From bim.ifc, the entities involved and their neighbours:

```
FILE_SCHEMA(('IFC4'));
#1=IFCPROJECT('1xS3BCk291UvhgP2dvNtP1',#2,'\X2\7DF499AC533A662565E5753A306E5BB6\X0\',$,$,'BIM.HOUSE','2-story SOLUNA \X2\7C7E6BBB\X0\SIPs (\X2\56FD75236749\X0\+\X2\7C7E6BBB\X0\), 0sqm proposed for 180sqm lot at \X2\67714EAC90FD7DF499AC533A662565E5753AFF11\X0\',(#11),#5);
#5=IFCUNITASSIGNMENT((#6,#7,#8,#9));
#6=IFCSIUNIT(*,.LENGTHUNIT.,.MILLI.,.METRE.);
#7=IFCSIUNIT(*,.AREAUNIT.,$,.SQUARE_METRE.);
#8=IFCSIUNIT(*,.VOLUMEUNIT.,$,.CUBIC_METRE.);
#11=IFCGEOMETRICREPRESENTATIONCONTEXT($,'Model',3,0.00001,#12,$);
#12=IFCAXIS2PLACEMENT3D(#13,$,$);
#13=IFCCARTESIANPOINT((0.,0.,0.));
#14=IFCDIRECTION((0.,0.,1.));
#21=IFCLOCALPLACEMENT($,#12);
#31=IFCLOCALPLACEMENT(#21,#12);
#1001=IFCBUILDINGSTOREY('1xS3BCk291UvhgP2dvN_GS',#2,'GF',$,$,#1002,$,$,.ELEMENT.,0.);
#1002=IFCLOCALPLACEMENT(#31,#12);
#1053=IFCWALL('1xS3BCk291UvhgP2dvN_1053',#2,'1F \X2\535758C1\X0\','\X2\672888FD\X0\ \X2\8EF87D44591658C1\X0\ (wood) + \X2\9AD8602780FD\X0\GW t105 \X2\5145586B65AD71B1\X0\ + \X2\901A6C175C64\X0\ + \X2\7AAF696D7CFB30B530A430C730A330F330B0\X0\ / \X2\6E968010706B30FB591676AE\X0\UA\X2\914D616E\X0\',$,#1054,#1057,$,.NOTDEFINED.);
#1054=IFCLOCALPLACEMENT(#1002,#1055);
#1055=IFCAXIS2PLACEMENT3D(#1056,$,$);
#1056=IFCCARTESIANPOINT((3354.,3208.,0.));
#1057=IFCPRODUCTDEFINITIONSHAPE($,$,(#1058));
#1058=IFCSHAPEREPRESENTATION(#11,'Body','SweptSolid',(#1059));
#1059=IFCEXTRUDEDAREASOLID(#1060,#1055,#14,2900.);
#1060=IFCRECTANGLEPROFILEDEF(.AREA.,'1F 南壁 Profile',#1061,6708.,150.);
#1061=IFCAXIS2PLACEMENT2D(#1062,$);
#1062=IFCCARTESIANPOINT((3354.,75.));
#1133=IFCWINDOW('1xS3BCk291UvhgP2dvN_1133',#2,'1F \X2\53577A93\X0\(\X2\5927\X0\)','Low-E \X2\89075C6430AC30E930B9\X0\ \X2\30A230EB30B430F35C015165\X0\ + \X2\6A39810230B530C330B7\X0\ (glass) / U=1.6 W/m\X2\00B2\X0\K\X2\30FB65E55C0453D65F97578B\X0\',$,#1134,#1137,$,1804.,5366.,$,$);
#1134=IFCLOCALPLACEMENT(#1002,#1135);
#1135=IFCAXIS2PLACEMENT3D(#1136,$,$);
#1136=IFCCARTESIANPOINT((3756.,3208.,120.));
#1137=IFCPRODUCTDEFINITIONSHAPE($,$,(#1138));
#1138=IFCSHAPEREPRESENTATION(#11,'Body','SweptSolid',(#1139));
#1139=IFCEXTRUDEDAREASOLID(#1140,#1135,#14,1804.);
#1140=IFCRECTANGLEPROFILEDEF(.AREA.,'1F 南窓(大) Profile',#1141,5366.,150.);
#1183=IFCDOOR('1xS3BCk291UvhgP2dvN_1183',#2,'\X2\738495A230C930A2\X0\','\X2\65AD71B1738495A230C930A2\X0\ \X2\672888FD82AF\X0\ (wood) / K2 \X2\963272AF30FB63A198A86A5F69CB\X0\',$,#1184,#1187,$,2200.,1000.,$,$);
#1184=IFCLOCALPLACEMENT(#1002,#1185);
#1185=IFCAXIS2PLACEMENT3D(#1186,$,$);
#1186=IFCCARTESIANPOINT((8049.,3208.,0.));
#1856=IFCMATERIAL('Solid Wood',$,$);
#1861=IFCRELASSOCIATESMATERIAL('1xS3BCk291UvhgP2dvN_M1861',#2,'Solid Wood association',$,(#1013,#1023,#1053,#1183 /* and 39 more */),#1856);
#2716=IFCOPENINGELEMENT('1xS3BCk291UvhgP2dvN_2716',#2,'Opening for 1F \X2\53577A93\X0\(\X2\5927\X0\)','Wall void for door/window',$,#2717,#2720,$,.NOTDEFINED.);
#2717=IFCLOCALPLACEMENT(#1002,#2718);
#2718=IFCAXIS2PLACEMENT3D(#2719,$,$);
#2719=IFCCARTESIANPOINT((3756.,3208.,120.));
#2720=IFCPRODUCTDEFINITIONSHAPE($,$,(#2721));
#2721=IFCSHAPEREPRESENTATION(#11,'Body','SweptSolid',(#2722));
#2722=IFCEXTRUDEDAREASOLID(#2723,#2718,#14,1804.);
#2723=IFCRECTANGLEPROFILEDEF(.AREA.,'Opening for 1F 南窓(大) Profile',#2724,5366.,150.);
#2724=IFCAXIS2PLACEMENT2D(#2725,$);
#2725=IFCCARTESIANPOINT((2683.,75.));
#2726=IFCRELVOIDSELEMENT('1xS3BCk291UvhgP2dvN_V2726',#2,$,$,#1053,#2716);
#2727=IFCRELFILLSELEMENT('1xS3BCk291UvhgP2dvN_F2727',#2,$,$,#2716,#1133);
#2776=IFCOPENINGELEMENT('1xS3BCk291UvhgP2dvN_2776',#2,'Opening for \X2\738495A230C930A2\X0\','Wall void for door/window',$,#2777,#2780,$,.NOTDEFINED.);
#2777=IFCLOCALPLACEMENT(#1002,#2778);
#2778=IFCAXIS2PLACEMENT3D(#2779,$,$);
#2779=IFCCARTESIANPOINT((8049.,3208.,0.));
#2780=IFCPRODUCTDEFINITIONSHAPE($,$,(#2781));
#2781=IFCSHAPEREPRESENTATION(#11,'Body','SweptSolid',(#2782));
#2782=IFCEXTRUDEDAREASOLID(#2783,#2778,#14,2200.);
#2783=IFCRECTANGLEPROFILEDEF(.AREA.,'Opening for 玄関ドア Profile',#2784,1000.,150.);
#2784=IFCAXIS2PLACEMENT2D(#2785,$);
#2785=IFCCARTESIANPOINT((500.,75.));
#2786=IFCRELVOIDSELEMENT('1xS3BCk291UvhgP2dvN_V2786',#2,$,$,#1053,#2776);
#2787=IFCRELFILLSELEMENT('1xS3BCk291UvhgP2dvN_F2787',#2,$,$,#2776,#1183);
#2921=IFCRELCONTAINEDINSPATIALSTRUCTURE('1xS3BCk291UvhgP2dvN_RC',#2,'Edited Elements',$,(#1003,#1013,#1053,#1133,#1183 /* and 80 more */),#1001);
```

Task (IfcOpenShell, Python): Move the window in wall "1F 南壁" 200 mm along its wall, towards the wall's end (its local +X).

```python
import ifcopenshell
import ifcopenshell.api.geometry
import ifcopenshell.util.placement
import ifcopenshell.util.unit

model = ifcopenshell.open("bim.ifc")
unit_scale = ifcopenshell.util.unit.calculate_unit_scale(model)

window = model.by_guid("1xS3BCk291UvhgP2dvN_1133")
opening = window.FillsVoids[0].RelatingOpeningElement
wall = opening.VoidsElements[0].RelatingBuildingElement

wall_matrix = ifcopenshell.util.placement.get_local_placement(wall.ObjectPlacement)
shift = wall_matrix[:3, 0] * 0.2 / unit_scale
before = ifcopenshell.util.placement.get_local_placement(window.ObjectPlacement)[:3, 3].copy()

# The window is not placed relative to its opening, so move both.
for product in (opening, window):
    matrix = ifcopenshell.util.placement.get_local_placement(product.ObjectPlacement)
    matrix[:3, 3] += shift
    ifcopenshell.api.geometry.edit_object_placement(model, product=product, matrix=matrix, is_si=False)

after = ifcopenshell.util.placement.get_local_placement(window.ObjectPlacement)[:3, 3]
print("window moved by", (after - before).round(3) + 0.0)

model.write("bim_edited.ifc")
```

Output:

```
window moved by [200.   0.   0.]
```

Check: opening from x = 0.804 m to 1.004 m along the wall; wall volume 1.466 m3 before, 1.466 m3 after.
